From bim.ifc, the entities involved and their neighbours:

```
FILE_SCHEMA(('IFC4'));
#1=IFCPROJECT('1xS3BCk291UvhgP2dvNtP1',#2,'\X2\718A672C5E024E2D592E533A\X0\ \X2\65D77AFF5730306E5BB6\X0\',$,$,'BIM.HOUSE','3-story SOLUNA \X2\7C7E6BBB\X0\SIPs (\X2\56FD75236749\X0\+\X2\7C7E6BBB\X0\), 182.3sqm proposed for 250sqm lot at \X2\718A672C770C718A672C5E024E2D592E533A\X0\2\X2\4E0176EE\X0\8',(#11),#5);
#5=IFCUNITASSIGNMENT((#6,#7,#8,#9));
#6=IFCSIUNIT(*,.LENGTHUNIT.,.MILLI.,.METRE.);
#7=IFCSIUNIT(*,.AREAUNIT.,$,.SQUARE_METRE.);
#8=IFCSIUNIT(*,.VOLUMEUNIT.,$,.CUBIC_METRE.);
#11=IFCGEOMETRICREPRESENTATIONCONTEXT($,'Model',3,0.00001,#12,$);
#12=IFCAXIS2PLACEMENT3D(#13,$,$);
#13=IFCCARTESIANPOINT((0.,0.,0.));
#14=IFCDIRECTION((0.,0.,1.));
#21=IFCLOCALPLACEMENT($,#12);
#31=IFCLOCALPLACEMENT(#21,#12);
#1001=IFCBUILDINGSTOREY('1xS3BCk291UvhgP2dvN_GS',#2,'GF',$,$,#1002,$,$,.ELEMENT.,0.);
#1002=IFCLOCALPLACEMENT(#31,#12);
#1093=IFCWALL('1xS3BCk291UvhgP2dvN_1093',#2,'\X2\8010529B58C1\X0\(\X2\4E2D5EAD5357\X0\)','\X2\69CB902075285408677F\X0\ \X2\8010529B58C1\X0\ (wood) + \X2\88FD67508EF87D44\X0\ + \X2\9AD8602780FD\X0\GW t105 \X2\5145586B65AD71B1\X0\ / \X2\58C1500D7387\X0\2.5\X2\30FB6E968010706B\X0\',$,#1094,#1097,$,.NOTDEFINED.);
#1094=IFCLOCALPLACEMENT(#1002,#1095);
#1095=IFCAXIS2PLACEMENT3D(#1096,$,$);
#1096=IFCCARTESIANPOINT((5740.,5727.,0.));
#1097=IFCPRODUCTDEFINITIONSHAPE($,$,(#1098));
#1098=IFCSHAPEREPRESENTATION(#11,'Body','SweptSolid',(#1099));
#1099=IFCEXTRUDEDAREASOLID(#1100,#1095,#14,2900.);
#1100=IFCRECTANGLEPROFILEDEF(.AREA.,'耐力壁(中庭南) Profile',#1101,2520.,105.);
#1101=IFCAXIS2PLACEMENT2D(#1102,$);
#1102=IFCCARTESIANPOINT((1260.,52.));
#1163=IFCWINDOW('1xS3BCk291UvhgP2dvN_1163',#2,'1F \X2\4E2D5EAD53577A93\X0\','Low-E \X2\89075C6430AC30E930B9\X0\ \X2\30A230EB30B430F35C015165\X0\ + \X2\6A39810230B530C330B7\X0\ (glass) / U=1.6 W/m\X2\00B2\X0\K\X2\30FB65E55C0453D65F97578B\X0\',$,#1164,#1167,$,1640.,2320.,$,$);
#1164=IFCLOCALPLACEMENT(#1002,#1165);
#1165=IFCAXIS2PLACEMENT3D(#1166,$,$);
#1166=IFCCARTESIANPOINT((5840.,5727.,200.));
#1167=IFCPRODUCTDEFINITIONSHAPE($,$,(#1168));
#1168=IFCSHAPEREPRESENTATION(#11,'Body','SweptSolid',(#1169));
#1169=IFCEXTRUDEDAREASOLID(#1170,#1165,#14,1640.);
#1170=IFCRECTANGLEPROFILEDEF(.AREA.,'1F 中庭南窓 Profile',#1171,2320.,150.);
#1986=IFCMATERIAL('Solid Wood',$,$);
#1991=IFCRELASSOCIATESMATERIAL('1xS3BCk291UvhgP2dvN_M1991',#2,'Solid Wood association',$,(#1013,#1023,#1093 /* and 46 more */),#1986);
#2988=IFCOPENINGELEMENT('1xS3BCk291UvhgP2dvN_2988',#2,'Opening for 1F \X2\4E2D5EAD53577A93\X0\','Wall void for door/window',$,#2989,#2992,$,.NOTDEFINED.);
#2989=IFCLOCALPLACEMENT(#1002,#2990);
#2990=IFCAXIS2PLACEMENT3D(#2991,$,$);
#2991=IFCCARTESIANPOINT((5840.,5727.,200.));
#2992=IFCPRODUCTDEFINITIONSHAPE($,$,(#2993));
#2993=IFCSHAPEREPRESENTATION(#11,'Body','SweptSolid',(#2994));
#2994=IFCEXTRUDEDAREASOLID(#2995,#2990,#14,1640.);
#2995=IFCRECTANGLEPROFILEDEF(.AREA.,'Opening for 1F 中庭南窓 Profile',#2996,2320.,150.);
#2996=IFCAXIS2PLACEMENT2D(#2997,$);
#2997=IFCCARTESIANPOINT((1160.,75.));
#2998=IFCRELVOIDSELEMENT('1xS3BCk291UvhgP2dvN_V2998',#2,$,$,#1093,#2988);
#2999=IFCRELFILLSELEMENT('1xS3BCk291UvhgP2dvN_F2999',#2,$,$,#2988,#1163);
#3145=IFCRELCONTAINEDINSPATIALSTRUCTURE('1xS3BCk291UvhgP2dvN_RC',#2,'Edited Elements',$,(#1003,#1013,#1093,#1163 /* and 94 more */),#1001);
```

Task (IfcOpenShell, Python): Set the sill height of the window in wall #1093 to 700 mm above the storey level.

```python
import numpy as np
import ifcopenshell
import ifcopenshell.api.geometry
import ifcopenshell.geom
import ifcopenshell.util.element
import ifcopenshell.util.placement
import ifcopenshell.util.shape
import ifcopenshell.util.unit

model = ifcopenshell.open("bim.ifc")
unit_scale = ifcopenshell.util.unit.calculate_unit_scale(model)

window = model.by_id(1163)
opening = window.FillsVoids[0].RelatingOpeningElement
storey = ifcopenshell.util.element.get_container(window, ifc_class="IfcBuildingStorey")
level = ifcopenshell.util.placement.get_local_placement(storey.ObjectPlacement)[2, 3]

# The opening's origin need not be at the sill, so measure its lowest point.
shape = ifcopenshell.geom.create_shape(ifcopenshell.geom.settings(), opening)
bottom = ifcopenshell.util.shape.get_shape_bottom_elevation(shape, shape.geometry) / unit_scale
dz = level + 700.0 - bottom

shift = np.array([0.0, 0.0, dz])
# The window is not placed relative to its opening, so move both.
for product in (opening, window):
    matrix = ifcopenshell.util.placement.get_local_placement(product.ObjectPlacement)
    matrix[:3, 3] += shift
    ifcopenshell.api.geometry.edit_object_placement(model, product=product, matrix=matrix, is_si=False)

print(f"moved by {dz * unit_scale:+.3f} m")

model.write("bim_edited.ifc")
```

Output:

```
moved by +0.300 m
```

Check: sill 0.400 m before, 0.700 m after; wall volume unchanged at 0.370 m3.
